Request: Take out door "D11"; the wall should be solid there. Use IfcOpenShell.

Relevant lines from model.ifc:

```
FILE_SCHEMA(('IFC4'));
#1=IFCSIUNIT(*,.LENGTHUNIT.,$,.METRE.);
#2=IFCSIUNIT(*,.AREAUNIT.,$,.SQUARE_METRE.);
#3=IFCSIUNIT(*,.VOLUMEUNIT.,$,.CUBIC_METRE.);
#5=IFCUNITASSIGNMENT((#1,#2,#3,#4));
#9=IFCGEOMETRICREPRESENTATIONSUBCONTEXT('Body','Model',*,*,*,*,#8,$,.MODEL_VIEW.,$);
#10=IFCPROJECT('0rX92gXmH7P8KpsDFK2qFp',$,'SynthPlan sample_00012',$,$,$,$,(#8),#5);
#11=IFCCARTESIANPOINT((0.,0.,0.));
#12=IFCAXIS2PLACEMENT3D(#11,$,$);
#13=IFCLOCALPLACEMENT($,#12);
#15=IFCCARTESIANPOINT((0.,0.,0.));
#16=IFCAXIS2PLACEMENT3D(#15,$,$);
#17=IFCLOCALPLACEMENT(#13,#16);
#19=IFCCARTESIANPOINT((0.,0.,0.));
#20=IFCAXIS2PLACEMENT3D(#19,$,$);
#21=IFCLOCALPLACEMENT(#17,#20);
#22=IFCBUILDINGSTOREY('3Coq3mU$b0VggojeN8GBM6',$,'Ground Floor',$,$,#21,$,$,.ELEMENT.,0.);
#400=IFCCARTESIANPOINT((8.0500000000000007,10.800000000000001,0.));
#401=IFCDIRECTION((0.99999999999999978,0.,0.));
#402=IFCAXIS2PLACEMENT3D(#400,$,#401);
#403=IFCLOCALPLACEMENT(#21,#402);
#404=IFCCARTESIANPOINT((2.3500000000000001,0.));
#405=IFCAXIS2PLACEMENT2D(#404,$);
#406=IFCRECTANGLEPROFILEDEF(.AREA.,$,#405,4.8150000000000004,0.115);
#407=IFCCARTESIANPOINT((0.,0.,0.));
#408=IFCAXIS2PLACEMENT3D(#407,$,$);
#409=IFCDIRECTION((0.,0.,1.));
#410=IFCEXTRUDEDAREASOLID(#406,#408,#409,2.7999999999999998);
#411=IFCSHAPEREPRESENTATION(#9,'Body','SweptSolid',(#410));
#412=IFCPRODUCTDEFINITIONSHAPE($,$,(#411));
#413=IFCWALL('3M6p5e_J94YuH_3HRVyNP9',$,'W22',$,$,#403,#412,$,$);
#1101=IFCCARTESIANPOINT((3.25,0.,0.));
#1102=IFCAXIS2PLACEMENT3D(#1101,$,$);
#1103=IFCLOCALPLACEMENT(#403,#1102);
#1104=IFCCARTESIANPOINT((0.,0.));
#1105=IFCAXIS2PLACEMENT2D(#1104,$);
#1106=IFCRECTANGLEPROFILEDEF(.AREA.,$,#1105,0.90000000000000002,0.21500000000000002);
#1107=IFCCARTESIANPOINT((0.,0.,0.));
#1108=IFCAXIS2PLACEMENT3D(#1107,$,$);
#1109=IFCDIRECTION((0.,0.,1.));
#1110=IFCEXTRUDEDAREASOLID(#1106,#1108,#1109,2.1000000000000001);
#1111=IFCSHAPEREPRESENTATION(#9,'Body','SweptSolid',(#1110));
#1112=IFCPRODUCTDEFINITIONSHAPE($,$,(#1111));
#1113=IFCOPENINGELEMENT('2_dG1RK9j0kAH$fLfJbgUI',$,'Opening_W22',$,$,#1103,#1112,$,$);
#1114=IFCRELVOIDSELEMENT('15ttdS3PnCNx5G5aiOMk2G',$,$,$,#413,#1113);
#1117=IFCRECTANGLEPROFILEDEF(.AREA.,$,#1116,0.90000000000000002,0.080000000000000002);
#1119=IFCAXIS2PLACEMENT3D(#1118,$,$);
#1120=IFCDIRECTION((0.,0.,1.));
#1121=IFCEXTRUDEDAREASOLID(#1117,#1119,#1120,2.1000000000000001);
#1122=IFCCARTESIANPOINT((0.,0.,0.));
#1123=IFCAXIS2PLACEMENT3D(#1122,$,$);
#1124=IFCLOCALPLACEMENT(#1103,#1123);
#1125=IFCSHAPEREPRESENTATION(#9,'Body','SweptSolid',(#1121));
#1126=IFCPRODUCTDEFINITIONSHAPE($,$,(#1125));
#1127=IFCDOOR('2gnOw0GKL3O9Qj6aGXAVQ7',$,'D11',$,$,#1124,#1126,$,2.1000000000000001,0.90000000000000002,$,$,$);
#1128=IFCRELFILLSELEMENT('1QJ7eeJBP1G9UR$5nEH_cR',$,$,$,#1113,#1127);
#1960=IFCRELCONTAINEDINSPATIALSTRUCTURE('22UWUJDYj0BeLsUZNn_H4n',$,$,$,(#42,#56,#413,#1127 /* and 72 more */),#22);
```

```python
import ifcopenshell
import ifcopenshell.api.feature
import ifcopenshell.api.root
import ifcopenshell.geom
import ifcopenshell.util.shape

model = ifcopenshell.open("model.ifc")
settings = ifcopenshell.geom.settings()


def volume(element):
    """Net volume in cubic metres, openings subtracted."""
    shape = ifcopenshell.geom.create_shape(settings, element)
    return ifcopenshell.util.shape.get_volume(shape.geometry)


door = model.by_id(1127)
opening = door.FillsVoids[0].RelatingOpeningElement
wall = opening.VoidsElements[0].RelatingBuildingElement
before = volume(wall)

ifcopenshell.api.root.remove_product(model, product=door)
ifcopenshell.api.feature.remove_feature(model, feature=opening)

after = volume(wall)

print(f"wall volume {before:.3f} -> {after:.3f} m3")

model.write("model_edited.ifc")
```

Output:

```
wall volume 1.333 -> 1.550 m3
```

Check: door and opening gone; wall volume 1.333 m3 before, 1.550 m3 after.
